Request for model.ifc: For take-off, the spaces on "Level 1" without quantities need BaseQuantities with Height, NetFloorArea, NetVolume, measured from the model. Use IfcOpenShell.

First a look at what the model holds.

```python
import ifcopenshell
import ifcopenshell.util.element
import ifcopenshell.util.unit

model = ifcopenshell.open("model.ifc")
print(model.schema)
for unit_type in ("LENGTHUNIT", "AREAUNIT", "VOLUMEUNIT"):
    print(unit_type, ifcopenshell.util.unit.calculate_unit_scale(model, unit_type))
storey = next(s for s in model.by_type("IfcBuildingStorey") if s.Name == "Level 1")
spaces = [e for e in ifcopenshell.util.element.get_decomposition(storey) if e.is_a("IfcSpace")]
for e in sorted(spaces, key=lambda e: e.id()):
    print(e.id(), e.is_a(), e.Name, list(ifcopenshell.util.element.get_psets(e, qtos_only=True)), sep=" | ")
```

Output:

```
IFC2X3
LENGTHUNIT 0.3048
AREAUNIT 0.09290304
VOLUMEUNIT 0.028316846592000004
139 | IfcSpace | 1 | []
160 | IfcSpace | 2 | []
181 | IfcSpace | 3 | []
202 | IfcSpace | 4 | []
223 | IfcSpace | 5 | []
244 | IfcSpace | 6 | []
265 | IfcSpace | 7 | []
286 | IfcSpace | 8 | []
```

```python
import ifcopenshell
import ifcopenshell.api.pset
import ifcopenshell.geom
import ifcopenshell.util.element
import ifcopenshell.util.shape
import ifcopenshell.util.unit

model = ifcopenshell.open("model.ifc")
unit_scale = ifcopenshell.util.unit.calculate_unit_scale(model)
area_scale = ifcopenshell.util.unit.calculate_unit_scale(model, "AREAUNIT")
volume_scale = ifcopenshell.util.unit.calculate_unit_scale(model, "VOLUMEUNIT")
settings = ifcopenshell.geom.settings()

storey = next(s for s in model.by_type("IfcBuildingStorey") if s.Name == "Level 1")
spaces = [e for e in ifcopenshell.util.element.get_decomposition(storey) if e.is_a("IfcSpace")]

for e in sorted(spaces, key=lambda e: e.id()):
    if ifcopenshell.util.element.get_psets(e, qtos_only=True, should_inherit=False):
        continue
    # Geometry comes back in metres, in the element's own axes.
    shape = ifcopenshell.geom.create_shape(settings, e)
    values = {
        "Height": ifcopenshell.util.shape.get_z(shape.geometry) / unit_scale,
        "NetFloorArea": ifcopenshell.util.shape.get_footprint_area(shape.geometry) / area_scale,
        "NetVolume": ifcopenshell.util.shape.get_volume(shape.geometry) / volume_scale,
    }
    qto = ifcopenshell.api.pset.add_qto(model, product=e, name="BaseQuantities")
    ifcopenshell.api.pset.edit_qto(model, qto=qto, properties=values)
    print(e.id(), {k: round(v, 3) for k, v in values.items()})

model.write("model_v2.ifc")
```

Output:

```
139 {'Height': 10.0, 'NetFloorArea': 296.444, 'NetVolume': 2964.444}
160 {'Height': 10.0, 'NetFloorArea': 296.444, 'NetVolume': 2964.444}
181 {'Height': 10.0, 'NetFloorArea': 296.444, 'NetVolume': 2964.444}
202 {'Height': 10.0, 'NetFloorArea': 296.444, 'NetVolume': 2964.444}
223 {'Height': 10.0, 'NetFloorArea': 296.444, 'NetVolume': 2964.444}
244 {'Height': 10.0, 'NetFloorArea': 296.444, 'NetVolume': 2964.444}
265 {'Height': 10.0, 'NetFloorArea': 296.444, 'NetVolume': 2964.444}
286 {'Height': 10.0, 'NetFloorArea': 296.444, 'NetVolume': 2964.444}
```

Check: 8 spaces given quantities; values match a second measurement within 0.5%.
